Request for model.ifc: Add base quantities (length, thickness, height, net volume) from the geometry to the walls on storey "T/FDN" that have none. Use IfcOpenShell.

First a look at what the model holds.

```python
import ifcopenshell
import ifcopenshell.util.element
import ifcopenshell.util.unit

model = ifcopenshell.open("model.ifc")
print(model.schema)
for unit_type in ("LENGTHUNIT", "AREAUNIT", "VOLUMEUNIT"):
    print(unit_type, ifcopenshell.util.unit.calculate_unit_scale(model, unit_type))
storey = next(s for s in model.by_type("IfcBuildingStorey") if s.Name == "T/FDN")
walls = [e for e in ifcopenshell.util.element.get_decomposition(storey) if e.is_a("IfcWall")]
for e in sorted(walls, key=lambda e: e.id()):
    print(e.id(), e.is_a(), e.Name, list(ifcopenshell.util.element.get_psets(e, qtos_only=True)), sep=" | ")
```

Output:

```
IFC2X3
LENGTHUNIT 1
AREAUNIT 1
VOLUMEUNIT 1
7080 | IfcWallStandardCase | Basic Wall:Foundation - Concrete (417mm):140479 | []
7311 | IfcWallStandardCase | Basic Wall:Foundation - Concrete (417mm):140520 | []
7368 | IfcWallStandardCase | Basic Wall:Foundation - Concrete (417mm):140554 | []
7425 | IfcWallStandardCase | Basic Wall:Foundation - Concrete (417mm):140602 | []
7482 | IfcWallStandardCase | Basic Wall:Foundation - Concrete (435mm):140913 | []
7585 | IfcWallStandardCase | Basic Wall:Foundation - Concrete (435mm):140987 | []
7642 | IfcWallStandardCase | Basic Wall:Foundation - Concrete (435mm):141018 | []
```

```python
import ifcopenshell
import ifcopenshell.api.pset
import ifcopenshell.geom
import ifcopenshell.util.element
import ifcopenshell.util.shape
import ifcopenshell.util.unit

model = ifcopenshell.open("model.ifc")
unit_scale = ifcopenshell.util.unit.calculate_unit_scale(model)
volume_scale = ifcopenshell.util.unit.calculate_unit_scale(model, "VOLUMEUNIT")
settings = ifcopenshell.geom.settings()

storey = next(s for s in model.by_type("IfcBuildingStorey") if s.Name == "T/FDN")
walls = [e for e in ifcopenshell.util.element.get_decomposition(storey) if e.is_a("IfcWall")]

for e in sorted(walls, key=lambda e: e.id()):
    if ifcopenshell.util.element.get_psets(e, qtos_only=True, should_inherit=False):
        continue
    # Geometry comes back in metres, in the element's own axes.
    shape = ifcopenshell.geom.create_shape(settings, e)
    values = {
        "Length": ifcopenshell.util.shape.get_x(shape.geometry) / unit_scale,
        "Width": ifcopenshell.util.shape.get_y(shape.geometry) / unit_scale,
        "Height": ifcopenshell.util.shape.get_z(shape.geometry) / unit_scale,
        "NetVolume": ifcopenshell.util.shape.get_volume(shape.geometry) / volume_scale,
    }
    qto = ifcopenshell.api.pset.add_qto(model, product=e, name="BaseQuantities")
    ifcopenshell.api.pset.edit_qto(model, qto=qto, properties=values)
    print(e.id(), {k: round(v, 3) for k, v in values.items()})

model.write("model_v2.ifc")
```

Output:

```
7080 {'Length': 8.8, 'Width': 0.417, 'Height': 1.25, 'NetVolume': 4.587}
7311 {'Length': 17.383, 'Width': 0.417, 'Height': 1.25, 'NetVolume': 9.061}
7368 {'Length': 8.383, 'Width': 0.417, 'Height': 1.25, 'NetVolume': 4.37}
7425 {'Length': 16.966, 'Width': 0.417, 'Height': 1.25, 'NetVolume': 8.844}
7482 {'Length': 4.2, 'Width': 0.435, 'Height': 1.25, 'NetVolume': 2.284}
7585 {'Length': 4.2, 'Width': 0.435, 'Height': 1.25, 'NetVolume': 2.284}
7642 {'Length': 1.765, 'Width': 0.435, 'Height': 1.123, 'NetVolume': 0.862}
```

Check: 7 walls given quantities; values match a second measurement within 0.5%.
